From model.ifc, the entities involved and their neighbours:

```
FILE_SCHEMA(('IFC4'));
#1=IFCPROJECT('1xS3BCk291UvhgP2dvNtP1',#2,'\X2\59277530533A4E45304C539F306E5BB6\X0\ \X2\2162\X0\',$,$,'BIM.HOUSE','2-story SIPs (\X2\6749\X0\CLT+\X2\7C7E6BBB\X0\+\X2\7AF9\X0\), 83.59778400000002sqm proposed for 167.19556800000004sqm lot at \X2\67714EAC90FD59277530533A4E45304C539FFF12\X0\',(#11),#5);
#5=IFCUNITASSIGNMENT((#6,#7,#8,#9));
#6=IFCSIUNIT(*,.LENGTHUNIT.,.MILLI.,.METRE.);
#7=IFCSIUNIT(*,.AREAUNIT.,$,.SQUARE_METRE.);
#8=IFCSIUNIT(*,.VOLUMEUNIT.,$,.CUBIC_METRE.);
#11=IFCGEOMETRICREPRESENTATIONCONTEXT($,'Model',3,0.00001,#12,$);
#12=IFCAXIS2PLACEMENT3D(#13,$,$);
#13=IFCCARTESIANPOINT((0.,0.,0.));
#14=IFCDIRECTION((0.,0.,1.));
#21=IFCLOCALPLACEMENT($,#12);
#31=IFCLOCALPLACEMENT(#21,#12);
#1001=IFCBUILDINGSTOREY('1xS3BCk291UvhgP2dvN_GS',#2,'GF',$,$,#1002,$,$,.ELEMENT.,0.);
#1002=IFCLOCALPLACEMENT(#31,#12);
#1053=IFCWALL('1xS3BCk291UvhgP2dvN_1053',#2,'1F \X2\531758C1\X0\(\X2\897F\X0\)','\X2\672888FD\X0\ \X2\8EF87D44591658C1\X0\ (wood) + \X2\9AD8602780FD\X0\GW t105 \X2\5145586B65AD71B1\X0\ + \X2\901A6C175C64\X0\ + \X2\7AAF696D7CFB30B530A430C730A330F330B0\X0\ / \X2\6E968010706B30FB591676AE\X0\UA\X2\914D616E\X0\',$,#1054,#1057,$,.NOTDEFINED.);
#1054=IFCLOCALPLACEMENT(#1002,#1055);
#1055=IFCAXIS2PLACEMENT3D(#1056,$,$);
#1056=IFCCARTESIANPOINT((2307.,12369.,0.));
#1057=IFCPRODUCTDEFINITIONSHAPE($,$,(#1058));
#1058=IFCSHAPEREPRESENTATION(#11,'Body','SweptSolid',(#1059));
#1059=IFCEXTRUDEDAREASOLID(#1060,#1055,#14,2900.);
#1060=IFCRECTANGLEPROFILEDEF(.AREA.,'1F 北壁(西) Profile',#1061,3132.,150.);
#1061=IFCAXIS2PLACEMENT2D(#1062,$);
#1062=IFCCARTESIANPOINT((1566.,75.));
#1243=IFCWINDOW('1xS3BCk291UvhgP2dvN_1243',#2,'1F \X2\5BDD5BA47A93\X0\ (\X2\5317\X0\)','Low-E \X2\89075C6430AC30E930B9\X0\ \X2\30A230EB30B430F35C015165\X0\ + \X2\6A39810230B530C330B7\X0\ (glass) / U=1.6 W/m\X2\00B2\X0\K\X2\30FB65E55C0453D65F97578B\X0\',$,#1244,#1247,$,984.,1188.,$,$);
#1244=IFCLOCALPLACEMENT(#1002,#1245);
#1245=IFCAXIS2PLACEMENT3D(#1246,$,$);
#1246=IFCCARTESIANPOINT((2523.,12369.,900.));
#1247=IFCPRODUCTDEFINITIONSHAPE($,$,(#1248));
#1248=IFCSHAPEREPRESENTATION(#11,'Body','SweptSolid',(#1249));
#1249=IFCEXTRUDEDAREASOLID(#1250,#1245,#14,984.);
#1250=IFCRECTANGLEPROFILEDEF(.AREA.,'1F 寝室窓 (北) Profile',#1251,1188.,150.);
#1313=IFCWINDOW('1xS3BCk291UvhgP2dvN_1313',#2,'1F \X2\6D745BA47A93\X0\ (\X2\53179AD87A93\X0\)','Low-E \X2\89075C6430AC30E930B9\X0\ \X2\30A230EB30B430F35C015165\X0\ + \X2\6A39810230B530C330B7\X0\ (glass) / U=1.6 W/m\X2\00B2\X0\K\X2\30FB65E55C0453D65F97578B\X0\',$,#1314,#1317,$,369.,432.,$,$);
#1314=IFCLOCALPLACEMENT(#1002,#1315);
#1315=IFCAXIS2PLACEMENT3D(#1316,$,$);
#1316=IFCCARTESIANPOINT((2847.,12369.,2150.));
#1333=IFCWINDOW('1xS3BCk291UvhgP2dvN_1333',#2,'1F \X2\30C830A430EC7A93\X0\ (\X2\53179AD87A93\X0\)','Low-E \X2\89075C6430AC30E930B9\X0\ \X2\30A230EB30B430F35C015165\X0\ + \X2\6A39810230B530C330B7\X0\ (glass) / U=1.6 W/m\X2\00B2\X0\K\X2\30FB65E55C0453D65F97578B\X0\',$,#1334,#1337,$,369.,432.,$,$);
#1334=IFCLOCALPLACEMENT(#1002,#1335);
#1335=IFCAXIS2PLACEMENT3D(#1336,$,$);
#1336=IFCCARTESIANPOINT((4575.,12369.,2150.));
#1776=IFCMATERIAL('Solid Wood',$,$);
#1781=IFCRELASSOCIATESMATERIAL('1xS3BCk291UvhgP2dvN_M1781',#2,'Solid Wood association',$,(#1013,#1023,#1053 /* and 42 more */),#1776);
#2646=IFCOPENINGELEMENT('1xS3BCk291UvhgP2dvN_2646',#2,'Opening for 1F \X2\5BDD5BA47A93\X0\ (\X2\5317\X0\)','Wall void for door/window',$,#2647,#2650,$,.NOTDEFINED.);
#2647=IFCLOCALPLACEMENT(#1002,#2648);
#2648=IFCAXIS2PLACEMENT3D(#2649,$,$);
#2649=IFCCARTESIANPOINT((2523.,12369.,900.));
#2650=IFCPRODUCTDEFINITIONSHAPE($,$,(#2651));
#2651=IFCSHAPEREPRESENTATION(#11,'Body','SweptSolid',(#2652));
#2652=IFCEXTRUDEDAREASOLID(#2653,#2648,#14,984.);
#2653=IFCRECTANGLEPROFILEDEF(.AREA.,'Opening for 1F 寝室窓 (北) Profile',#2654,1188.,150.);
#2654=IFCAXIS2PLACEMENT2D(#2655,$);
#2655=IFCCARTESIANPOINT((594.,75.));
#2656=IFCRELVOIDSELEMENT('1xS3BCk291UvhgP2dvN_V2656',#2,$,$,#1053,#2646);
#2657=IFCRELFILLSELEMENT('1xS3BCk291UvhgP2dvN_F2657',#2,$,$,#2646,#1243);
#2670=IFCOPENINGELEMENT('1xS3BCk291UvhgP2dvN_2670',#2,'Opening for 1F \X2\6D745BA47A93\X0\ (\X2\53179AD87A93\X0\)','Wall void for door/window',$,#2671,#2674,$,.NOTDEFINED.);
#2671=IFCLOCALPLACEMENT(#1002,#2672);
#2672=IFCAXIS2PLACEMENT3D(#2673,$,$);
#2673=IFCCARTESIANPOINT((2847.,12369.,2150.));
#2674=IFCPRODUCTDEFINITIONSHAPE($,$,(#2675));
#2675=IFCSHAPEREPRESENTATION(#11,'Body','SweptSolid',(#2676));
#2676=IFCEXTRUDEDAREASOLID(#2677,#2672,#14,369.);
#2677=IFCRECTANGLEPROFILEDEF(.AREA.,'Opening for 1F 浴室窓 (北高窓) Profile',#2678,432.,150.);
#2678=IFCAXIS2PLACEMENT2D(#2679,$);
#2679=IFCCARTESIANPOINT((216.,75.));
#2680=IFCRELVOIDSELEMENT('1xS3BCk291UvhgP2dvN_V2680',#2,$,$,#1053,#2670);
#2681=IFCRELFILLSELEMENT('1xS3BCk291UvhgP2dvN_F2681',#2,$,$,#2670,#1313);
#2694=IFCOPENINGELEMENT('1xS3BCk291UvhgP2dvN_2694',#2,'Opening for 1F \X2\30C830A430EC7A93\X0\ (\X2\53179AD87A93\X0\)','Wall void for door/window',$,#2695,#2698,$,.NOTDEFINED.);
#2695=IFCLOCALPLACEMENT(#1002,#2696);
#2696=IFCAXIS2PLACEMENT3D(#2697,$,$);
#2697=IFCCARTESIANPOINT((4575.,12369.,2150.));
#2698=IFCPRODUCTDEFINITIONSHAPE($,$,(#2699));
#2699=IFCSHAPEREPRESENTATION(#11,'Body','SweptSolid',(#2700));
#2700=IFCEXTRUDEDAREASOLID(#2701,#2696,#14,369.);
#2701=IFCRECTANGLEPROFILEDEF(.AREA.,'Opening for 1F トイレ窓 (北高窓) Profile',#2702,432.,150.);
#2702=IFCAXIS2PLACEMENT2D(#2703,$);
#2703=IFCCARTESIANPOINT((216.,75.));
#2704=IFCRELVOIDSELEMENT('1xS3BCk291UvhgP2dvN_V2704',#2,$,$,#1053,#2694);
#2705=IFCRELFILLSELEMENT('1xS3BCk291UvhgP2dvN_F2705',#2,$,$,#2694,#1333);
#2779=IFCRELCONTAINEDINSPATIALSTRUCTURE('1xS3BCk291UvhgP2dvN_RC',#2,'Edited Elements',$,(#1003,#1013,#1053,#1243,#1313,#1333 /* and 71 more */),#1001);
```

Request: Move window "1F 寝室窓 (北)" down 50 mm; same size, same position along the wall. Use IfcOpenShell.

```python
import numpy as np
import ifcopenshell
import ifcopenshell.api.geometry
import ifcopenshell.util.placement
import ifcopenshell.util.unit

model = ifcopenshell.open("model.ifc")
unit_scale = ifcopenshell.util.unit.calculate_unit_scale(model)

window = model.by_id(1243)
opening = window.FillsVoids[0].RelatingOpeningElement
dz = -50.0

shift = np.array([0.0, 0.0, dz])
# The window is not placed relative to its opening, so move both.
for product in (opening, window):
    matrix = ifcopenshell.util.placement.get_local_placement(product.ObjectPlacement)
    matrix[:3, 3] += shift
    ifcopenshell.api.geometry.edit_object_placement(model, product=product, matrix=matrix, is_si=False)

print(f"moved by {dz * unit_scale:+.3f} m")

model.write("model-out.ifc")
```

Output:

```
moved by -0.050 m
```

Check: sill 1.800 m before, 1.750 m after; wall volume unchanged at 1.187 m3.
